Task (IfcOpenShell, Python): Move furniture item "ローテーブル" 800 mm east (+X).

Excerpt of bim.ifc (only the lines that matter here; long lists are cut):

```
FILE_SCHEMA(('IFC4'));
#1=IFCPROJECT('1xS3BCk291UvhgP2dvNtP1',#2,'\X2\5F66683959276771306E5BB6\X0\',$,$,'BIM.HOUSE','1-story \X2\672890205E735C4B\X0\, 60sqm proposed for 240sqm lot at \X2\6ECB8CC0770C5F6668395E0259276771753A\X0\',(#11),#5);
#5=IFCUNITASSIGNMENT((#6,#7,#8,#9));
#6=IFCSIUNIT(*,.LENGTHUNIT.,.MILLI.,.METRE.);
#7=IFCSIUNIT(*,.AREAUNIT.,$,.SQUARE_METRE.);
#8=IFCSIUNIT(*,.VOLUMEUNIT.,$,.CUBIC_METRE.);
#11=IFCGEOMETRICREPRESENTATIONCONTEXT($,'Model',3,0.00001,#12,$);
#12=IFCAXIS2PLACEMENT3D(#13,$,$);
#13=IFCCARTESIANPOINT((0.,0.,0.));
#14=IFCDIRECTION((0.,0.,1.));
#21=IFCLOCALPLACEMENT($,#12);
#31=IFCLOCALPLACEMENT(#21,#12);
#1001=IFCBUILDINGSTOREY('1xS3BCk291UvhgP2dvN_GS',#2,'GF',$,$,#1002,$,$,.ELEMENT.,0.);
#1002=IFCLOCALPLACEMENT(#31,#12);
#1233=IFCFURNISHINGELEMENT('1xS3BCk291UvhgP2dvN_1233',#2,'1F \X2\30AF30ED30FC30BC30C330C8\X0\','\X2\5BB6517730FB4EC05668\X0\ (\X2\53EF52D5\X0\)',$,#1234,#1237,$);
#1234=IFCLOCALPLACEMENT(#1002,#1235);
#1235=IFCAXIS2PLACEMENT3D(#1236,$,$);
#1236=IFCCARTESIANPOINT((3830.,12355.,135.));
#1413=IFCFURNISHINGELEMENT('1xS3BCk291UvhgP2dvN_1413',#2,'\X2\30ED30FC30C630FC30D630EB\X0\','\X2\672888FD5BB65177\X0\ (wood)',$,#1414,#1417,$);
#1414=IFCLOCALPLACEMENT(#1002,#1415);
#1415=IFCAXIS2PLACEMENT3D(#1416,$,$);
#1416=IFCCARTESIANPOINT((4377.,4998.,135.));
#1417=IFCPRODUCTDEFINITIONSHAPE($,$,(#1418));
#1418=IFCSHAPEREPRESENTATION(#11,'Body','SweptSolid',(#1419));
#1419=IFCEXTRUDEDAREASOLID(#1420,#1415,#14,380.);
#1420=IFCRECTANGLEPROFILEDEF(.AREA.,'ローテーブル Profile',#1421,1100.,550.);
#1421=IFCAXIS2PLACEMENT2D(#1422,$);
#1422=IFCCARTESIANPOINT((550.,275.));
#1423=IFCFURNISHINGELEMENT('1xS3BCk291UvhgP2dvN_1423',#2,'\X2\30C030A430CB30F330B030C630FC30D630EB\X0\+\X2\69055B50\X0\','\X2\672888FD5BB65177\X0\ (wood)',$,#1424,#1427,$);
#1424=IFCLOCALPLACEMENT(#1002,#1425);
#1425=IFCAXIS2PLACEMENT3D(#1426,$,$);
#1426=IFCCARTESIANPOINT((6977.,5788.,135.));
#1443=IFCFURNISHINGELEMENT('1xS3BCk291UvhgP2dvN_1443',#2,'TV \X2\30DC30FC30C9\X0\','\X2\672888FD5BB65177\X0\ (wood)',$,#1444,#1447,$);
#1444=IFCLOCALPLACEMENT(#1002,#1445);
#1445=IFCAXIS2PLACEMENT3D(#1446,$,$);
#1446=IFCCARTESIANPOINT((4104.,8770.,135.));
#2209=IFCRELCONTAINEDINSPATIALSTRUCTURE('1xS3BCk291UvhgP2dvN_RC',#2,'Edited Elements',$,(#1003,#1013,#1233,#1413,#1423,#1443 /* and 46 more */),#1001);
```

```python
import ifcopenshell
import ifcopenshell.api.geometry
import ifcopenshell.util.placement

model = ifcopenshell.open("bim.ifc")

item = model.by_guid("1xS3BCk291UvhgP2dvN_1413")
matrix = ifcopenshell.util.placement.get_local_placement(item.ObjectPlacement)
matrix[0, 3] += 800.0
ifcopenshell.api.geometry.edit_object_placement(model, product=item, matrix=matrix, is_si=False)

print(ifcopenshell.util.placement.get_local_placement(item.ObjectPlacement).round(3) + 0.0)

model.write("bim_updated.ifc")
```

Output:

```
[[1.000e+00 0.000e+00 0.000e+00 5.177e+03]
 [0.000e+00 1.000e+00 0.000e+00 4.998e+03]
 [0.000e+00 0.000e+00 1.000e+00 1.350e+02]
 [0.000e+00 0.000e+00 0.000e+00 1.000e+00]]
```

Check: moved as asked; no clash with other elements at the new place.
